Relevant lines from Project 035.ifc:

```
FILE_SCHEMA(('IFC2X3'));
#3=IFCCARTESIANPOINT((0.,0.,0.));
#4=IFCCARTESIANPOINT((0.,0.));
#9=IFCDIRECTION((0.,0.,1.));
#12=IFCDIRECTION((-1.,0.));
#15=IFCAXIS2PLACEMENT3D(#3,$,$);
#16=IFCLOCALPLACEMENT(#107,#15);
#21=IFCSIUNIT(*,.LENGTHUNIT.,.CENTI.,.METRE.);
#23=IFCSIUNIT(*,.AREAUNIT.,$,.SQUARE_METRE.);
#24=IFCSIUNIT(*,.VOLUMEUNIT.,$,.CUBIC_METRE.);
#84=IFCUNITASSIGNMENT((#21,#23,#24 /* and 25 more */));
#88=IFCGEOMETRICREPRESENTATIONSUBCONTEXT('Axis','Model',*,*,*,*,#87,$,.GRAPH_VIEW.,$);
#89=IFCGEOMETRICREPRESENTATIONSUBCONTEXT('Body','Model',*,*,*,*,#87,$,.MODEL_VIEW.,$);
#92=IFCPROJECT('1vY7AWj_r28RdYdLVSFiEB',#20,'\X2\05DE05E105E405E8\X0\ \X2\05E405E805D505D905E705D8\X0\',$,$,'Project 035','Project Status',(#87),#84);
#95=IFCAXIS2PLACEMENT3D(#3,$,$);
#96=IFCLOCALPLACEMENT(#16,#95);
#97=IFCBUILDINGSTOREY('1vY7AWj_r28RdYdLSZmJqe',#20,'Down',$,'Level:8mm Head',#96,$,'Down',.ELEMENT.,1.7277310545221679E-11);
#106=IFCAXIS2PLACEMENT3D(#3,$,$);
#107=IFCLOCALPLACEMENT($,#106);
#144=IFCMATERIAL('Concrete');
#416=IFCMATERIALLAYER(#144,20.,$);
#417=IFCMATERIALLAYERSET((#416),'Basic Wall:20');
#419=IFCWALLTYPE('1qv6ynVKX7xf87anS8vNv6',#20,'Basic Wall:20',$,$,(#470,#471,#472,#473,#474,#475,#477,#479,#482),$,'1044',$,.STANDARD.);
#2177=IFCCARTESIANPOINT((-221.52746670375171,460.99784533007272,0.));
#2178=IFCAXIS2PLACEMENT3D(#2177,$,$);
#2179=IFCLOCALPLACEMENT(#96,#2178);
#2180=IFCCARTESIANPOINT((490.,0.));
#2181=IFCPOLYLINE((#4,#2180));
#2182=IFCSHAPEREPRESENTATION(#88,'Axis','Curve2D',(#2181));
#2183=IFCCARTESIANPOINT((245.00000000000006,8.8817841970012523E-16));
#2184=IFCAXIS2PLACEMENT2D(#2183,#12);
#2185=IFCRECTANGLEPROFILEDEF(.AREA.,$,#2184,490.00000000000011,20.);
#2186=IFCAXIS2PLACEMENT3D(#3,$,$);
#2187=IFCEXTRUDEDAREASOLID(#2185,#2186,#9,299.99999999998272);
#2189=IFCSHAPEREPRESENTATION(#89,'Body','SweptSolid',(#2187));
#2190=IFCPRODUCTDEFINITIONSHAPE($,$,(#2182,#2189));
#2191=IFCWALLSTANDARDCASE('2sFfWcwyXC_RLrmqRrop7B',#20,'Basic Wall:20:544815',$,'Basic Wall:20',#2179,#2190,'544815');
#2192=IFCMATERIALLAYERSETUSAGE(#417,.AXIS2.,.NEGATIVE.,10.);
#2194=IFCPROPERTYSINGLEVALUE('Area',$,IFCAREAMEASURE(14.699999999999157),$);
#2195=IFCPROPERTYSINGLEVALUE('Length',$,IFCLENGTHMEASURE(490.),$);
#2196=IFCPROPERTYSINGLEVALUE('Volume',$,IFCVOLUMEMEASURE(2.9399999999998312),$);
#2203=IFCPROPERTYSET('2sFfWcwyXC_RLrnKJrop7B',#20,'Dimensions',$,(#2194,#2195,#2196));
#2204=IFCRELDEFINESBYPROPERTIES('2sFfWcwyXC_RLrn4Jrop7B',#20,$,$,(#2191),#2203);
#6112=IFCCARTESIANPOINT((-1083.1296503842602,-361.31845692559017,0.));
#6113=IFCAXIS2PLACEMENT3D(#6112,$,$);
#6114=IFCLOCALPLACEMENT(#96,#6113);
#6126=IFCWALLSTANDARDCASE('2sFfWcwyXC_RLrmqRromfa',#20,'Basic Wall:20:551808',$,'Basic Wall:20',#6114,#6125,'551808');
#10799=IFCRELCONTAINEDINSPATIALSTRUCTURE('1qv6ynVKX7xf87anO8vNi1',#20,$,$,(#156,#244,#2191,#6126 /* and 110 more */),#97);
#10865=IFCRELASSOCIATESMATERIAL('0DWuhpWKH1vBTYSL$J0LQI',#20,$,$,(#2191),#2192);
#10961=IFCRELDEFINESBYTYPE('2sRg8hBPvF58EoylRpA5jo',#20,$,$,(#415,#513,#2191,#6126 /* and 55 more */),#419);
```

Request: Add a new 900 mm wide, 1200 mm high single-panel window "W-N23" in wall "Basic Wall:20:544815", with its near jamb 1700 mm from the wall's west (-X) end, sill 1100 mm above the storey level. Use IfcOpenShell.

```python
import numpy as np
import ifcopenshell
import ifcopenshell.api.feature
import ifcopenshell.api.geometry
import ifcopenshell.api.pset
import ifcopenshell.api.root
import ifcopenshell.api.spatial
import ifcopenshell.api.type
import ifcopenshell.geom
import ifcopenshell.util.element
import ifcopenshell.util.placement
import ifcopenshell.util.representation
import ifcopenshell.util.shape
import ifcopenshell.util.unit

model = ifcopenshell.open("Project 035.ifc")
unit_scale = ifcopenshell.util.unit.calculate_unit_scale(model)
area_scale = ifcopenshell.util.unit.calculate_unit_scale(model, "AREAUNIT")
volume_scale = ifcopenshell.util.unit.calculate_unit_scale(model, "VOLUMEUNIT")
settings = ifcopenshell.geom.settings()


def volume(element):
    """Net volume in cubic metres, openings subtracted."""
    shape = ifcopenshell.geom.create_shape(settings, element)
    return ifcopenshell.util.shape.get_volume(shape.geometry)


wall = model.by_guid("2sFfWcwyXC_RLrmqRrop7B")
storey = ifcopenshell.util.element.get_container(wall, ifc_class="IfcBuildingStorey")
context = ifcopenshell.util.representation.get_context(model, "Model", "Body", "MODEL_VIEW")
before = volume(wall)

width, height, from_end, sill = 0.9, 1.2, 1.7, 1.1  # metres

# The wall runs along its own X axis, and the end named is its -X end.
wall_shape = ifcopenshell.geom.create_shape(settings, wall)
x, y, z = ifcopenshell.util.shape.get_vertices(wall_shape.geometry).T
start = x.min() + from_end
face, thickness = float(y.min()), float(y.max() - y.min())
wall_matrix = ifcopenshell.util.placement.get_local_placement(wall.ObjectPlacement)
level = ifcopenshell.util.placement.get_local_placement(storey.ObjectPlacement)[2, 3]


def in_wall(x, y):
    """Placement at x, y metres in the wall's axes, at sill height."""
    matrix = wall_matrix.copy()
    matrix[:, 3] = wall_matrix @ np.array([x / unit_scale, y / unit_scale, 0.0, 1.0])
    matrix[2, 3] = level + sill / unit_scale
    return matrix


# Opening: a box that overshoots both wall faces by 50 mm.
opening = ifcopenshell.api.root.create_entity(model, ifc_class="IfcOpeningElement")
box = ifcopenshell.api.geometry.add_wall_representation(
    model, context=context, length=width, height=height, thickness=thickness + 0.1
)
ifcopenshell.api.geometry.assign_representation(model, product=opening, representation=box)
ifcopenshell.api.geometry.edit_object_placement(model, product=opening, matrix=in_wall(start, face - 0.05), is_si=False)
ifcopenshell.api.feature.add_feature(model, feature=opening, element=wall)

window = ifcopenshell.api.root.create_entity(model, ifc_class="IfcWindow", name="W-N23")
window.OverallWidth, window.OverallHeight = width / unit_scale, height / unit_scale
body = ifcopenshell.api.geometry.add_window_representation(
    model,
    context=context,
    overall_width=window.OverallWidth,
    overall_height=window.OverallHeight,
    partition_type="SINGLE_PANEL",
)
ifcopenshell.api.geometry.assign_representation(model, product=window, representation=body)
ifcopenshell.api.spatial.assign_container(model, products=[window], relating_structure=storey)
fills = ifcopenshell.api.feature.add_filling(model, opening=opening, element=window)
fills.OwnerHistory = window.OwnerHistory  # required in IFC2X3

# IFC2X3 keeps the operation on the window style.
style = ifcopenshell.api.root.create_entity(model, ifc_class="IfcWindowStyle", name="W-N23")
style.OperationType, style.ConstructionType = "SINGLE_PANEL", "NOTDEFINED"
style.ParameterTakesPrecedence = style.Sizeable = False
ifcopenshell.api.type.assign_type(model, related_objects=[window], relating_type=style)

# Centre the window in the wall's thickness.
ifcopenshell.api.geometry.edit_object_placement(model, product=window, matrix=in_wall(start, face), is_si=False)
window_shape = ifcopenshell.geom.create_shape(settings, window)
depth = ifcopenshell.util.shape.get_vertices(window_shape.geometry)[:, 1]
offset = face + thickness / 2 - (depth.min() + depth.max()) / 2
ifcopenshell.api.geometry.edit_object_placement(model, product=window, matrix=in_wall(start, offset), is_si=False)

after = volume(wall)

# Update the wall's stored quantities.
pset = model.by_id(ifcopenshell.util.element.get_pset(wall, "Dimensions", should_inherit=False)["id"])
ifcopenshell.api.pset.edit_pset(model, pset=pset, properties={
    "Area": model.create_entity("IfcAreaMeasure", after / thickness / area_scale),
    "Volume": model.create_entity("IfcVolumeMeasure", after / volume_scale),
})

print(f"wall volume {before:.3f} -> {after:.3f} m3")

model.write("Project 035_edited.ifc")
```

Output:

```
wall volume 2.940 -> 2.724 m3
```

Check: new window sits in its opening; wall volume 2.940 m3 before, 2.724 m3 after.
